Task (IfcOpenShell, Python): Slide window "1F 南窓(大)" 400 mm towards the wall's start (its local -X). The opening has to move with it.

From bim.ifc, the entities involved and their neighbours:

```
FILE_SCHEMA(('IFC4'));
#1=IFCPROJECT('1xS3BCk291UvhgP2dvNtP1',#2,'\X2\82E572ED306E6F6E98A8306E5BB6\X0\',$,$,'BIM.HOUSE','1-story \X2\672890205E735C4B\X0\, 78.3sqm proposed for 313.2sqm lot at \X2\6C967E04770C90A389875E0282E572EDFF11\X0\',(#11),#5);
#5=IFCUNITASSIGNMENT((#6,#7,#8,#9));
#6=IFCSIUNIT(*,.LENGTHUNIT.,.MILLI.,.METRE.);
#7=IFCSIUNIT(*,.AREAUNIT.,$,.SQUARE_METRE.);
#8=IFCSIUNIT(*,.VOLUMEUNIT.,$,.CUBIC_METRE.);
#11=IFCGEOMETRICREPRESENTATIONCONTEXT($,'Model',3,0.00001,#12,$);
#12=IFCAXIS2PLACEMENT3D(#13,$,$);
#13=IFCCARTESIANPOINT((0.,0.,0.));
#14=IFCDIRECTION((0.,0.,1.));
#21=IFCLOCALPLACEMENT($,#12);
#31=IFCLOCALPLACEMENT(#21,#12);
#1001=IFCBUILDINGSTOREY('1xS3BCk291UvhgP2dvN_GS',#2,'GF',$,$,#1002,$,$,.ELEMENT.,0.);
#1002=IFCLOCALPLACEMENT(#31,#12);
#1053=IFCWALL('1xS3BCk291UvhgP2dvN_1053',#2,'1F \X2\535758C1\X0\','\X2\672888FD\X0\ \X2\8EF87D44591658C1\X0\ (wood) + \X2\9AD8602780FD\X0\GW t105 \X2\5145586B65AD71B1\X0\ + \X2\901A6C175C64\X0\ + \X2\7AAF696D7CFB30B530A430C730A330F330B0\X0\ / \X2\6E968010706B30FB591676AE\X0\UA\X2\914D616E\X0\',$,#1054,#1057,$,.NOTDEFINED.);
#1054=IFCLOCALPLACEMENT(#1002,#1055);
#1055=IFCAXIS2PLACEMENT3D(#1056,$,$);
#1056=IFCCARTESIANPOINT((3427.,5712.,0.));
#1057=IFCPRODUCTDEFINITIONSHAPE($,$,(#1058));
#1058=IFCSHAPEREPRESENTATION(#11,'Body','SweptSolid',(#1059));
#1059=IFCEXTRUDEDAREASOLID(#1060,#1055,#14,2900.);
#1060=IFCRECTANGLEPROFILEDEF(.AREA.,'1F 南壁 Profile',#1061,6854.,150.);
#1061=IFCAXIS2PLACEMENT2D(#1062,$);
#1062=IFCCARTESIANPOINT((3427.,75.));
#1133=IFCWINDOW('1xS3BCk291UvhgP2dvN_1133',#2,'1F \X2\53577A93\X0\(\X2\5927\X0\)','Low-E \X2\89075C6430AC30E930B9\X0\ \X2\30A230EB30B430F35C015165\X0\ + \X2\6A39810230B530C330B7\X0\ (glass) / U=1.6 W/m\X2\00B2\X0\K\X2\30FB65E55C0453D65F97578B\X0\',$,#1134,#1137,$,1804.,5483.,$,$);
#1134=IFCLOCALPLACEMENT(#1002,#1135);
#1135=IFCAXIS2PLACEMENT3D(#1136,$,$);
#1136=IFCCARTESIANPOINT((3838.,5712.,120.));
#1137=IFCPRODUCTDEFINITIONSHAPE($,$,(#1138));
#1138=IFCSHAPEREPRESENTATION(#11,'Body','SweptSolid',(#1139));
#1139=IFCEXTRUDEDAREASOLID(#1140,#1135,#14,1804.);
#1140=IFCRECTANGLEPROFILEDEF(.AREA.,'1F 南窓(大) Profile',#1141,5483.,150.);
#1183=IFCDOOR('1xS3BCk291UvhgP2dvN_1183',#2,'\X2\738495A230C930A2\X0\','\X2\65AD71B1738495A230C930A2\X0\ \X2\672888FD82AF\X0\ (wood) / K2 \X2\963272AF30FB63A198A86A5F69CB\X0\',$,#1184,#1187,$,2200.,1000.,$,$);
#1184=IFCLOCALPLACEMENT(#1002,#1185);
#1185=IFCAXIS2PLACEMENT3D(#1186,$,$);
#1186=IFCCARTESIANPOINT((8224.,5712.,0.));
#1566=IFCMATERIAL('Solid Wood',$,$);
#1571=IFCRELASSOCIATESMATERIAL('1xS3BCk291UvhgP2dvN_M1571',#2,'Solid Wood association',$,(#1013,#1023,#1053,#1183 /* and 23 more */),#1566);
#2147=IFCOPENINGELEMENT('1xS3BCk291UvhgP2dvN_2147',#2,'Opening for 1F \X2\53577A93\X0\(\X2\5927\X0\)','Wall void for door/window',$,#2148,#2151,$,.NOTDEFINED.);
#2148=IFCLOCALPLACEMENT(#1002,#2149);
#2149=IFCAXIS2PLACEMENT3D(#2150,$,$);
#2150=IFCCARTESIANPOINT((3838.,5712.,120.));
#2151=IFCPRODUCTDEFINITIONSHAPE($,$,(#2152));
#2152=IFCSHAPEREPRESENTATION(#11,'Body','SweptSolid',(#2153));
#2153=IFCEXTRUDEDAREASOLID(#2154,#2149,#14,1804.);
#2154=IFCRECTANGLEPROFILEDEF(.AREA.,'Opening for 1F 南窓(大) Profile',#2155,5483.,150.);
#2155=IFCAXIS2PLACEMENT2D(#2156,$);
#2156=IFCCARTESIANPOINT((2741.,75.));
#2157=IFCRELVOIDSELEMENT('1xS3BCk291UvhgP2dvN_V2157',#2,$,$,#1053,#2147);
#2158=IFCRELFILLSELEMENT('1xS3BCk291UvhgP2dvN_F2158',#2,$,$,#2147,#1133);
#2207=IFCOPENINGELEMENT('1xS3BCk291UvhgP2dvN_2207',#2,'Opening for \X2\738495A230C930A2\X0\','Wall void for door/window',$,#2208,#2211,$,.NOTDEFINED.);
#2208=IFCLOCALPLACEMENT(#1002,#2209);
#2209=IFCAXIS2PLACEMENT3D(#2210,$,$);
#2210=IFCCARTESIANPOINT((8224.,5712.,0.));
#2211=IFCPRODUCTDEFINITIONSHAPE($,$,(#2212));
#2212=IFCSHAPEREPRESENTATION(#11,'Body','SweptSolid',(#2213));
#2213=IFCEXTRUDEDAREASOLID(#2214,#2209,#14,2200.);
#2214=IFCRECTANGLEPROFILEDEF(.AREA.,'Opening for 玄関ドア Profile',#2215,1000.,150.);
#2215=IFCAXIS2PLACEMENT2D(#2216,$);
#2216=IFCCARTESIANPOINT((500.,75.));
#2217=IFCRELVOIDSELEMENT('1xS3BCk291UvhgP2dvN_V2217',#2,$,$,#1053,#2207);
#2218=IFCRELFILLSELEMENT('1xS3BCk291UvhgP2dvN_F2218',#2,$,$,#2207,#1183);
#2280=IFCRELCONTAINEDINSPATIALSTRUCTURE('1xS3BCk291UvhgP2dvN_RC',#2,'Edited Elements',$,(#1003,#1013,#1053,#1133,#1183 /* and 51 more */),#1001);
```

```python
import ifcopenshell
import ifcopenshell.api.geometry
import ifcopenshell.util.placement
import ifcopenshell.util.unit

model = ifcopenshell.open("bim.ifc")
unit_scale = ifcopenshell.util.unit.calculate_unit_scale(model)

window = model.by_guid("1xS3BCk291UvhgP2dvN_1133")
opening = window.FillsVoids[0].RelatingOpeningElement
wall = opening.VoidsElements[0].RelatingBuildingElement

wall_matrix = ifcopenshell.util.placement.get_local_placement(wall.ObjectPlacement)
shift = wall_matrix[:3, 0] * -0.4 / unit_scale
before = ifcopenshell.util.placement.get_local_placement(window.ObjectPlacement)[:3, 3].copy()

# The window is not placed relative to its opening, so move both.
for product in (opening, window):
    matrix = ifcopenshell.util.placement.get_local_placement(product.ObjectPlacement)
    matrix[:3, 3] += shift
    ifcopenshell.api.geometry.edit_object_placement(model, product=product, matrix=matrix, is_si=False)

after = ifcopenshell.util.placement.get_local_placement(window.ObjectPlacement)[:3, 3]
print("window moved by", (after - before).round(3) + 0.0)

model.write("bim_updated.ifc")
```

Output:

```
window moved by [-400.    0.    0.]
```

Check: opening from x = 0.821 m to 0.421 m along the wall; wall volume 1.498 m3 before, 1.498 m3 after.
